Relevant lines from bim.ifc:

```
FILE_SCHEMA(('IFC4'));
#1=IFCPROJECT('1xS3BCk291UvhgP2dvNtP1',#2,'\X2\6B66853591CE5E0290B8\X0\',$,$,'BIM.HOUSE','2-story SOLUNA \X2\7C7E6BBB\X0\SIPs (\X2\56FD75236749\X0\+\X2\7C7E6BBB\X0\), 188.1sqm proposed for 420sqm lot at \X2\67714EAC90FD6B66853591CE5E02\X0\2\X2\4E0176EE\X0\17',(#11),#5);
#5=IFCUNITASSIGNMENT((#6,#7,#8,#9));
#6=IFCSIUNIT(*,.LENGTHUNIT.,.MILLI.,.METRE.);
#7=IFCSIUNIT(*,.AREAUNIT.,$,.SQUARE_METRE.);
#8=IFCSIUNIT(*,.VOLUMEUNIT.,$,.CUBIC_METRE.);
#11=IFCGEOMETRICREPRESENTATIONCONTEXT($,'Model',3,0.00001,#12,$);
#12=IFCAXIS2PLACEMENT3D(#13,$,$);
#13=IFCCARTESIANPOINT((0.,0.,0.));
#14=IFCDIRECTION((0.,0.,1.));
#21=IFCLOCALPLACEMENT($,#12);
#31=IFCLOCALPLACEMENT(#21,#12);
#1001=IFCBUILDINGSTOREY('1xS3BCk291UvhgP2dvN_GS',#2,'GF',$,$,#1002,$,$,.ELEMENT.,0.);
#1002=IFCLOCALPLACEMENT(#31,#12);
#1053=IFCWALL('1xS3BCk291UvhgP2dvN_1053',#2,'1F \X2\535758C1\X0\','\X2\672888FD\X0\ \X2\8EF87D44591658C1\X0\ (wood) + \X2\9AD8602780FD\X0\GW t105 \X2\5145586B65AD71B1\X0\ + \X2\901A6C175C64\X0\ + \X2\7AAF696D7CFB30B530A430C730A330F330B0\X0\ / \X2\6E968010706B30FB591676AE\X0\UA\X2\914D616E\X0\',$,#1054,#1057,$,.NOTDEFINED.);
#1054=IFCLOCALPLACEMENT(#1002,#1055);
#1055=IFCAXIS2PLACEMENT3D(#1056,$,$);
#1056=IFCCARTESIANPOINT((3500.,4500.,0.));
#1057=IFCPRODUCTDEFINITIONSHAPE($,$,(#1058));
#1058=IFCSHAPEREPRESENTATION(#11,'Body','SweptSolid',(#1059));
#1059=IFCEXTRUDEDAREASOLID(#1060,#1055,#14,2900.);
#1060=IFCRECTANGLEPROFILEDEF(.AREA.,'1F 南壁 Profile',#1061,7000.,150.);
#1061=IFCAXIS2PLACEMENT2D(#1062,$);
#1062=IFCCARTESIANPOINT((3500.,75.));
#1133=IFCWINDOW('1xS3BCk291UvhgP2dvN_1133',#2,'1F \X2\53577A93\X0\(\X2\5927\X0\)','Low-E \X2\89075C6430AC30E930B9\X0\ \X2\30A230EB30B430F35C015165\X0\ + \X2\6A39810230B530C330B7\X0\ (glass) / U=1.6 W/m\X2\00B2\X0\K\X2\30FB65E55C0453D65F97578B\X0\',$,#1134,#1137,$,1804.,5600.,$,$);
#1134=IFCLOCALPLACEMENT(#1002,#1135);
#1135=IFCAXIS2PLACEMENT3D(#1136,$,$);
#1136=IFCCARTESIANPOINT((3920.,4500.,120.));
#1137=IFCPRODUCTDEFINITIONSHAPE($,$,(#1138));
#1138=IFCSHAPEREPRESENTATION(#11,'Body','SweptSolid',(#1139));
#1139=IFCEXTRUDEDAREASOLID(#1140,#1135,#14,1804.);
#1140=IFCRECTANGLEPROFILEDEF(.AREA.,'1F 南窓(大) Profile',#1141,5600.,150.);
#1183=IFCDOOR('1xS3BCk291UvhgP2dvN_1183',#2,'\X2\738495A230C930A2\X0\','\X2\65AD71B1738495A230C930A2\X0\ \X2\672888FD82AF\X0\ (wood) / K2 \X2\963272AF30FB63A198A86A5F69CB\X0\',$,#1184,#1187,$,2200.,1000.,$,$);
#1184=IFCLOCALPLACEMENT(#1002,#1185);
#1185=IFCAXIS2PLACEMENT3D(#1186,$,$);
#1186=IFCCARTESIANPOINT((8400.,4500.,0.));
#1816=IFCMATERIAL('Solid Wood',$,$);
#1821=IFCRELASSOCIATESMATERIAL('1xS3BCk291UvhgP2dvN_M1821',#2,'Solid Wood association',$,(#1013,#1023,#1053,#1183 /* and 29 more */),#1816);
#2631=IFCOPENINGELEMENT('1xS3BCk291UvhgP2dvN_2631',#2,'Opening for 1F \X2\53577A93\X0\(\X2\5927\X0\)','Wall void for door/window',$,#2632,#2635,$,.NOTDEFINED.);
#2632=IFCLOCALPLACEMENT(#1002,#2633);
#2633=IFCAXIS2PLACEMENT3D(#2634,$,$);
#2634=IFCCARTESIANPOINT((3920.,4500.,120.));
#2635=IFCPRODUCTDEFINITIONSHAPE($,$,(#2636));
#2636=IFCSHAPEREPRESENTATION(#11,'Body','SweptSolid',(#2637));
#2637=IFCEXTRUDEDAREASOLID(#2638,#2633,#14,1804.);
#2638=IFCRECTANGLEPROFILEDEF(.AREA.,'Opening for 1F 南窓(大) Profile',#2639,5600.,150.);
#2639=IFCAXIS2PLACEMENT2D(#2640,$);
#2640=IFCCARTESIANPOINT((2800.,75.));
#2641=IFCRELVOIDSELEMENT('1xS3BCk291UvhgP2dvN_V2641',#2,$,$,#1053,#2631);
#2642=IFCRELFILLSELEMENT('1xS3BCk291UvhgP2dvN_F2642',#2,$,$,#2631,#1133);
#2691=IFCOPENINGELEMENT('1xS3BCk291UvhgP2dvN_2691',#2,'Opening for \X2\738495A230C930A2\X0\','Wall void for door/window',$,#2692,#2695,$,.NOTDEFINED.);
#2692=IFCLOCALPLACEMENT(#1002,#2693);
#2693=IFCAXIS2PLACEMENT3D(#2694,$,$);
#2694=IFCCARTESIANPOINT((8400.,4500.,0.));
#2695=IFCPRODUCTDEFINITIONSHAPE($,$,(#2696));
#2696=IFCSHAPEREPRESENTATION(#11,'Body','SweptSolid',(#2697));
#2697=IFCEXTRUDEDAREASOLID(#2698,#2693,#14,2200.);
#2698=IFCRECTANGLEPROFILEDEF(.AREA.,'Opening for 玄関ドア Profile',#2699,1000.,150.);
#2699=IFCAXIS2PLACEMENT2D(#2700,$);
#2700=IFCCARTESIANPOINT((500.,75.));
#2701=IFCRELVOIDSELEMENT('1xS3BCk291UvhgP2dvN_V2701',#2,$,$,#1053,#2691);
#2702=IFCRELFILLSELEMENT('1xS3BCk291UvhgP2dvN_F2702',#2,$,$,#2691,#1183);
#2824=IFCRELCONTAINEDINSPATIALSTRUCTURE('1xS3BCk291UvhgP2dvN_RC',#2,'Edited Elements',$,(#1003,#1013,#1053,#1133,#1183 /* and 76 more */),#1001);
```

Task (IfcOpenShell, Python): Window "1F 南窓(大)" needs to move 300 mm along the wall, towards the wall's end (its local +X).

```python
import ifcopenshell
import ifcopenshell.api.geometry
import ifcopenshell.util.placement
import ifcopenshell.util.unit

model = ifcopenshell.open("bim.ifc")
unit_scale = ifcopenshell.util.unit.calculate_unit_scale(model)

window = model.by_id(1133)
opening = window.FillsVoids[0].RelatingOpeningElement
wall = opening.VoidsElements[0].RelatingBuildingElement

wall_matrix = ifcopenshell.util.placement.get_local_placement(wall.ObjectPlacement)
shift = wall_matrix[:3, 0] * 0.3 / unit_scale
before = ifcopenshell.util.placement.get_local_placement(window.ObjectPlacement)[:3, 3].copy()

# The window is not placed relative to its opening, so move both.
for product in (opening, window):
    matrix = ifcopenshell.util.placement.get_local_placement(product.ObjectPlacement)
    matrix[:3, 3] += shift
    ifcopenshell.api.geometry.edit_object_placement(model, product=product, matrix=matrix, is_si=False)

after = ifcopenshell.util.placement.get_local_placement(window.ObjectPlacement)[:3, 3]
print("window moved by", (after - before).round(3) + 0.0)

model.write("bim_edited.ifc")
```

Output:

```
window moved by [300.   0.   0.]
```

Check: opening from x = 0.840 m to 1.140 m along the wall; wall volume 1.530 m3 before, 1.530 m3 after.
